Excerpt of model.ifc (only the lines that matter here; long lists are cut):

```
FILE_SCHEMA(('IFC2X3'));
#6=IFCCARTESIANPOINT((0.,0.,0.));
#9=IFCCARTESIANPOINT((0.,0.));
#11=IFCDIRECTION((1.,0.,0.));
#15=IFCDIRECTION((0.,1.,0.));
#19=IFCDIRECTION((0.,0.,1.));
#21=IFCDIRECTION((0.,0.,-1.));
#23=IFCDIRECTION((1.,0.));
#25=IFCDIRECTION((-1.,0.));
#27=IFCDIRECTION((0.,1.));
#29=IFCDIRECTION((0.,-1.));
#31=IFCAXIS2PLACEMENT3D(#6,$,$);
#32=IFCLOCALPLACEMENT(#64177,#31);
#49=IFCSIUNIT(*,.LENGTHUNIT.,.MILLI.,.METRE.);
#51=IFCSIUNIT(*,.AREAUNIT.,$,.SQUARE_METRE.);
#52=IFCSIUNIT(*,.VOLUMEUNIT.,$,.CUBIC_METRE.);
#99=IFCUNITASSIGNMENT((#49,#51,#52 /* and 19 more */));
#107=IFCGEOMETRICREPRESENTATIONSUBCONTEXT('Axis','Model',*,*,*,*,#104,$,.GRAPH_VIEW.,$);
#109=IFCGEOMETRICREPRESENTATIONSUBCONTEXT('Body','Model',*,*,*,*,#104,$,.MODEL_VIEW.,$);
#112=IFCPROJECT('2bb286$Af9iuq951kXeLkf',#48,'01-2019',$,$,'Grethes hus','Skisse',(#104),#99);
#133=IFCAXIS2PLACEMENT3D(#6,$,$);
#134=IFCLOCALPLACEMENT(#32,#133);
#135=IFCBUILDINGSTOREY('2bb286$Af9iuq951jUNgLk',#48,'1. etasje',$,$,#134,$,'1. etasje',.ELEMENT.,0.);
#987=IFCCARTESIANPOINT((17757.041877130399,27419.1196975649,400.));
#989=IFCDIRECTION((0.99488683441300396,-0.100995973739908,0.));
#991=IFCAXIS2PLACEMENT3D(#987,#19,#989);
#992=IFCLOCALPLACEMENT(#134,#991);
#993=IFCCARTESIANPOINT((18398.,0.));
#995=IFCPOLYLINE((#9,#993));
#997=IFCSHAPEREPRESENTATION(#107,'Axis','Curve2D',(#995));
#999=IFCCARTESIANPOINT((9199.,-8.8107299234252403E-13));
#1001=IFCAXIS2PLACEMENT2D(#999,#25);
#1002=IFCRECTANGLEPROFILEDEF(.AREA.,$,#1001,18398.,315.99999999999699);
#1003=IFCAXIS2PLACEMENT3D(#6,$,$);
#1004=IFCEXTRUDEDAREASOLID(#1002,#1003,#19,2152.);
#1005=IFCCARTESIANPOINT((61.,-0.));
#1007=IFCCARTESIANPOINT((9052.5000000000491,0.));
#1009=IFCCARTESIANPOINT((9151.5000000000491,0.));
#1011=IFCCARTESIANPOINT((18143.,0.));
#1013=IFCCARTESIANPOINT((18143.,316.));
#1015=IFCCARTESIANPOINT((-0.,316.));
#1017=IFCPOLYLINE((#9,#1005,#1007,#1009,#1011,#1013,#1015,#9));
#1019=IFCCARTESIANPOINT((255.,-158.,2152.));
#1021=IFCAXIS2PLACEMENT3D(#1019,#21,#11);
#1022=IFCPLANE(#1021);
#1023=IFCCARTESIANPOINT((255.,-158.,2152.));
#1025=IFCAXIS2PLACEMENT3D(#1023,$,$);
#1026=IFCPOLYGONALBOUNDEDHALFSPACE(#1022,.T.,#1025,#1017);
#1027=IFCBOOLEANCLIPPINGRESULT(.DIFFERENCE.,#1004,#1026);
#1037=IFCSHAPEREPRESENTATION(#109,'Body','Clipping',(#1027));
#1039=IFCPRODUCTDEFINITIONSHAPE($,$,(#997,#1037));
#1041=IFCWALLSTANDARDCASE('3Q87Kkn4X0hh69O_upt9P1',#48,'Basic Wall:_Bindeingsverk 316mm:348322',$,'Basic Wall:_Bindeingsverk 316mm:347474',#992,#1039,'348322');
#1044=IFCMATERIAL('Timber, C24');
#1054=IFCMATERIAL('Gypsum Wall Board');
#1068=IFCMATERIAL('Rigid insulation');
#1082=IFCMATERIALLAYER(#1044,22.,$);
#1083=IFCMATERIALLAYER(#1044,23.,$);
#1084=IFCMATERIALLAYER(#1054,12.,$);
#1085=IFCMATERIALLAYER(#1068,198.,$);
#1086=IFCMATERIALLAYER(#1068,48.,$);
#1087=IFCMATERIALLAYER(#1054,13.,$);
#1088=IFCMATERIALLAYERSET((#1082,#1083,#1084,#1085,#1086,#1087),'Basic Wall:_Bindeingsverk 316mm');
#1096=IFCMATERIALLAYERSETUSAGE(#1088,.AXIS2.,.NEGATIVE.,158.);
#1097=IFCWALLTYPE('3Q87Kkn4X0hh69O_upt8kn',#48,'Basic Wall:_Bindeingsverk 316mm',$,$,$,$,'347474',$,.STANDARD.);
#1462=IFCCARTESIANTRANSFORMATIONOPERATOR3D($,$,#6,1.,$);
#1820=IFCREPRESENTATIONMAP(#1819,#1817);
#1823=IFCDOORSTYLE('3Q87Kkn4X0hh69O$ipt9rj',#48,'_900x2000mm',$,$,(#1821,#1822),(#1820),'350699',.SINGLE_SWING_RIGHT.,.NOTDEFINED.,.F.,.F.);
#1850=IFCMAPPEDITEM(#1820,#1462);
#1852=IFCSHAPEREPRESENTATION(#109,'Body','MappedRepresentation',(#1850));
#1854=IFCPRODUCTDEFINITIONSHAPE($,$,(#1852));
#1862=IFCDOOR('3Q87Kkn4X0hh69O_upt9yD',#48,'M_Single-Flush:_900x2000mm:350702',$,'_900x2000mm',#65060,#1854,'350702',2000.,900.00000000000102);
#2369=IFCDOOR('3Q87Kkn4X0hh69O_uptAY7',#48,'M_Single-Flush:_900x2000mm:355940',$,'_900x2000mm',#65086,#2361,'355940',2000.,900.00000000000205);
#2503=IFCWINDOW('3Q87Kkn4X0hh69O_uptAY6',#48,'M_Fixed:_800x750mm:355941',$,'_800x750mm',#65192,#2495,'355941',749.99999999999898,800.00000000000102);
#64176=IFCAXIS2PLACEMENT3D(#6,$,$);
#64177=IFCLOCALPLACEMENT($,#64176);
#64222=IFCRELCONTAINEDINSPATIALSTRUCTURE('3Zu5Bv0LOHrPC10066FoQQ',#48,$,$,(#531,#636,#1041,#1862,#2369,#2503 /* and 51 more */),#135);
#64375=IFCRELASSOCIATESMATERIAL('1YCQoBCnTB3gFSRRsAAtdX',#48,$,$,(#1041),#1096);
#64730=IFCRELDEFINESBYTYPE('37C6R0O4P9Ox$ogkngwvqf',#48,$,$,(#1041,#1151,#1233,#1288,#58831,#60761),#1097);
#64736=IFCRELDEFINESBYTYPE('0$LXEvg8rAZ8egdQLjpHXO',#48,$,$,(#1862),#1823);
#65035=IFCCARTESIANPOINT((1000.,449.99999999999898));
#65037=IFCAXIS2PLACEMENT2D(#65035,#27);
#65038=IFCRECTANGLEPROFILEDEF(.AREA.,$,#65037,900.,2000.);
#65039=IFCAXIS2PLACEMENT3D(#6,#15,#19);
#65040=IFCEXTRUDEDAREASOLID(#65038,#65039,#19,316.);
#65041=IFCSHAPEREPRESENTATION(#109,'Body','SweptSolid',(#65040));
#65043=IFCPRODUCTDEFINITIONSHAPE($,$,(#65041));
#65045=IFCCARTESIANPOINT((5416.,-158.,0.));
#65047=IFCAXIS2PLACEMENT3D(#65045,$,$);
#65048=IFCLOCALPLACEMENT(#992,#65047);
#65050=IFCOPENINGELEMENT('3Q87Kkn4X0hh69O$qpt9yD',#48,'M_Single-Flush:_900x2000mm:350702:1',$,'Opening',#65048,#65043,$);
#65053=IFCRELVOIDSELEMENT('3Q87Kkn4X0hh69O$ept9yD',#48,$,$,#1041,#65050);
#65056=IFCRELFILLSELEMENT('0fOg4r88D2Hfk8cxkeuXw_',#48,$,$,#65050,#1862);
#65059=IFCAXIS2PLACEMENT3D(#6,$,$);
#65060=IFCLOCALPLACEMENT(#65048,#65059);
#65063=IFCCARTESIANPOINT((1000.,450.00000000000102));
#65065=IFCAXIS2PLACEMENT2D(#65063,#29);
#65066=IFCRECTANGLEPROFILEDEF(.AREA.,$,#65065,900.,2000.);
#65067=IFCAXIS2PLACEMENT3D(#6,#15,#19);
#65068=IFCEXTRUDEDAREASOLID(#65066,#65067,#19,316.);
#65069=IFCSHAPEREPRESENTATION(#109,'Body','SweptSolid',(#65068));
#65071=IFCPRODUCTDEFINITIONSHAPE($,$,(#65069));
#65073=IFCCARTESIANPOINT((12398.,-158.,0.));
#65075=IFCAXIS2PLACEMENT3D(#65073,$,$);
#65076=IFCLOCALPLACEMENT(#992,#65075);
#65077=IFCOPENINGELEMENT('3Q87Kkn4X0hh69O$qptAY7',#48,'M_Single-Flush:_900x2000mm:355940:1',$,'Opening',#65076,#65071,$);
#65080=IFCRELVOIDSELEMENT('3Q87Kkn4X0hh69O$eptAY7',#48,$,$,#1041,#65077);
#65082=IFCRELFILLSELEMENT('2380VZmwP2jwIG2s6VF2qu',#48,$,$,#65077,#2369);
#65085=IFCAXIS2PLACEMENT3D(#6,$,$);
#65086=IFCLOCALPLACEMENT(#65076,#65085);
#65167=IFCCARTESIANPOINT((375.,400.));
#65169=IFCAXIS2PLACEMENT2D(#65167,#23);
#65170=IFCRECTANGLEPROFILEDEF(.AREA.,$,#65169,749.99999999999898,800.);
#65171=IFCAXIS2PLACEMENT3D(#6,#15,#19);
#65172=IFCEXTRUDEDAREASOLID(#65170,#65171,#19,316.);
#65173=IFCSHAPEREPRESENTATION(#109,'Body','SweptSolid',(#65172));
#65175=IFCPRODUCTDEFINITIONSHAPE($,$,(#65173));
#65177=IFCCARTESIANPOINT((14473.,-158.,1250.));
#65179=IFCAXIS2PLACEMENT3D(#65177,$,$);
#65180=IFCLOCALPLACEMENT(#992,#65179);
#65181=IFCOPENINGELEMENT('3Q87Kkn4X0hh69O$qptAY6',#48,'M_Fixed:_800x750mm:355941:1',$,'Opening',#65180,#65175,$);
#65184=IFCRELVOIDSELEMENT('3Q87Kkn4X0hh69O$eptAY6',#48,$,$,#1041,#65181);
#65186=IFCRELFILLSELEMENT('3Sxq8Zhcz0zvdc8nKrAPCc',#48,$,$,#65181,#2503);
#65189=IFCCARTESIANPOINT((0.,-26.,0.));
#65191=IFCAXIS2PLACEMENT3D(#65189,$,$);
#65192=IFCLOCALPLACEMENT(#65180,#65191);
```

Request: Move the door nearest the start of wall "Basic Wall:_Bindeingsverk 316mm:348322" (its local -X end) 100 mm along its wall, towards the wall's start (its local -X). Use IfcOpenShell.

```python
import ifcopenshell
import ifcopenshell.api.geometry
import ifcopenshell.util.placement

model = ifcopenshell.open("model.ifc")

door = model.by_guid("3Q87Kkn4X0hh69O_upt9yD")
opening = door.FillsVoids[0].RelatingOpeningElement
wall = opening.VoidsElements[0].RelatingBuildingElement

wall_matrix = ifcopenshell.util.placement.get_local_placement(wall.ObjectPlacement)
shift = wall_matrix[:3, 0] * -100.0
before = ifcopenshell.util.placement.get_local_placement(door.ObjectPlacement)[:3, 3].copy()

# The door is placed relative to its opening, so it follows when the opening moves.
matrix = ifcopenshell.util.placement.get_local_placement(opening.ObjectPlacement)
matrix[:3, 3] += shift
ifcopenshell.api.geometry.edit_object_placement(
    model, product=opening, matrix=matrix, is_si=False, should_transform_children=True
)

after = ifcopenshell.util.placement.get_local_placement(door.ObjectPlacement)[:3, 3]
print("door moved by", (after - before).round(3) + 0.0)

model.write("model_edited.ifc")
```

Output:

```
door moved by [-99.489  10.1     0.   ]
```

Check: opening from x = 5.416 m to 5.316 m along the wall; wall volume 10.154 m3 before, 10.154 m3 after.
